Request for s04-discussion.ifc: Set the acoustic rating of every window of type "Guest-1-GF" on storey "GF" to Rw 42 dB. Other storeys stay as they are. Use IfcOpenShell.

First a look at what the model holds.

```python
import ifcopenshell
import ifcopenshell.util.element

model = ifcopenshell.open("s04-discussion.ifc")
print(model.schema)
storey = next(s for s in model.by_type("IfcBuildingStorey") if s.Name == "GF")
windows = [e for e in ifcopenshell.util.element.get_decomposition(storey) if e.is_a("IfcWindow")]
seen = {}
for e in windows:
    element_type = ifcopenshell.util.element.get_type(e)
    key = (element_type.Name if element_type != e and element_type else None, ifcopenshell.util.element.get_pset(e, "Pset_WindowCommon", "AcousticRating"))
    seen[key] = seen.get(key, 0) + 1
for (name, value), count in sorted(seen.items(), key=str):
    print(count, "x", name, "|", value)
```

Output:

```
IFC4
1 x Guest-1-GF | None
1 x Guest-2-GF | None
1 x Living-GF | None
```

```python
import ifcopenshell
import ifcopenshell.api.pset
import ifcopenshell.util.element

model = ifcopenshell.open("s04-discussion.ifc")

storey = next(s for s in model.by_type("IfcBuildingStorey") if s.Name == "GF")
windows = [e for e in ifcopenshell.util.element.get_decomposition(storey) if e.is_a("IfcWindow")]

count = 0
for e in windows:
    element_type = ifcopenshell.util.element.get_type(e)
    if element_type in (None, e) or element_type.Name != "Guest-1-GF":
        continue
    # add_pset returns the element's existing set when there is one.
    pset = ifcopenshell.api.pset.add_pset(model, product=e, name="Pset_WindowCommon")
    ifcopenshell.api.pset.edit_pset(model, pset=pset, properties={"AcousticRating": "Rw 42 dB"})
    count += 1

print(count, "windows updated")

model.write("s04-discussion_rev.ifc")
```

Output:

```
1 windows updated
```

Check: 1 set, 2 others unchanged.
